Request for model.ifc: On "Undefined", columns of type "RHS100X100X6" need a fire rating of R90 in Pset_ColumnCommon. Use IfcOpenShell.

First a look at what the model holds.

```python
import ifcopenshell
import ifcopenshell.util.element

model = ifcopenshell.open("model.ifc")
print(model.schema)
storey = next(s for s in model.by_type("IfcBuildingStorey") if s.Name == "Undefined")
columns = [e for e in ifcopenshell.util.element.get_decomposition(storey) if e.is_a("IfcColumn")]
seen = {}
for e in columns:
    element_type = ifcopenshell.util.element.get_type(e)
    key = (element_type.Name if element_type != e and element_type else None, ifcopenshell.util.element.get_pset(e, "Pset_ColumnCommon", "FireRating"))
    seen[key] = seen.get(key, 0) + 1
for (name, value), count in sorted(seen.items(), key=str):
    print(count, "x", name, "|", value)
```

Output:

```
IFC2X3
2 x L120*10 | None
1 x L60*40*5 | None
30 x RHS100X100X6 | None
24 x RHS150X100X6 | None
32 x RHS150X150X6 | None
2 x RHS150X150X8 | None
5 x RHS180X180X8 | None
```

```python
import ifcopenshell
import ifcopenshell.api.pset
import ifcopenshell.util.element

model = ifcopenshell.open("model.ifc")

storey = next(s for s in model.by_type("IfcBuildingStorey") if s.Name == "Undefined")
columns = [e for e in ifcopenshell.util.element.get_decomposition(storey) if e.is_a("IfcColumn")]

count = 0
for e in columns:
    element_type = ifcopenshell.util.element.get_type(e)
    if element_type in (None, e) or element_type.Name != "RHS100X100X6":
        continue
    found = ifcopenshell.util.element.get_pset(e, "Pset_ColumnCommon", should_inherit=False)
    if found:
        pset = model.by_id(found["id"])
        if len(ifcopenshell.util.element.get_elements_by_pset(pset)) > 1:
            pset = ifcopenshell.api.pset.unshare_pset(model, products=[e], pset=pset)[0]
    else:
        pset = ifcopenshell.api.pset.add_pset(model, product=e, name="Pset_ColumnCommon")
    ifcopenshell.api.pset.edit_pset(model, pset=pset, properties={"FireRating": "R90"})
    count += 1

print(count, "columns updated")

model.write("model_v2.ifc")
```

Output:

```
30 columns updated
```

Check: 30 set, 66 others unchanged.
